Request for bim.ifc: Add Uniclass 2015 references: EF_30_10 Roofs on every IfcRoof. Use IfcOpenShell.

First a look at what the model holds.

```python
import ifcopenshell

model = ifcopenshell.open("bim.ifc")
print(model.schema)
print("classifications:", [c.Name for c in model.by_type("IfcClassification")])
for ifc_class in ("IfcDoor", "IfcRoof", "IfcStair", "IfcWall", "IfcWindow"):
    print(ifc_class, len(model.by_type(ifc_class)))
```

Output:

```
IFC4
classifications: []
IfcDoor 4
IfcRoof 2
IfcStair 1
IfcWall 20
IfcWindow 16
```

```python
import ifcopenshell
import ifcopenshell.api.classification

model = ifcopenshell.open("bim.ifc")

system = ifcopenshell.api.classification.add_classification(model, classification="Uniclass 2015")

codes = {
    "IfcRoof": ("EF_30_10", "Roofs"),
}
for ifc_class, (code, name) in codes.items():
    products = model.by_type(ifc_class)
    ifcopenshell.api.classification.add_reference(
        model, products=products, classification=system, identification=code, name=name
    )
    print(code, len(products))

model.write("bim_rev.ifc")
```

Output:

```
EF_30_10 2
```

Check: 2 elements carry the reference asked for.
